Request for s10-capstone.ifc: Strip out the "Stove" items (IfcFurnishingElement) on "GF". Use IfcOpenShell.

First a look at what the model holds.

```python
import ifcopenshell
import ifcopenshell.util.element

model = ifcopenshell.open("s10-capstone.ifc")
print(model.schema)
storey = next(s for s in model.by_type("IfcBuildingStorey") if s.Name == "GF")
furniture = [e for e in ifcopenshell.util.element.get_decomposition(storey) if e.is_a("IfcFurnishingElement")]
seen = {}
for e in furniture:
    element_type = ifcopenshell.util.element.get_type(e)
    name = element_type.Name if element_type not in (None, e) else None
    seen[name] = seen.get(name, 0) + 1
for name, count in sorted(seen.items(), key=str):
    print(count, "x", name)
```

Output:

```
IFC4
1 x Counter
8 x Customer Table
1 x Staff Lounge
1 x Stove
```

```python
import ifcopenshell
import ifcopenshell.api.root
import ifcopenshell.util.element

model = ifcopenshell.open("s10-capstone.ifc")

storey = next(s for s in model.by_type("IfcBuildingStorey") if s.Name == "GF")
furniture = [e for e in ifcopenshell.util.element.get_decomposition(storey) if e.is_a("IfcFurnishingElement")]
targets = [e for e in furniture if (t := ifcopenshell.util.element.get_type(e)) not in (None, e) and t.Name == "Stove"]

for e in targets:
    ifcopenshell.api.root.remove_product(model, product=e)
print(len(targets), "removed")

model.write("s10-capstone_rev.ifc")
```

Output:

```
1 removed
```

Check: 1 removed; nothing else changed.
